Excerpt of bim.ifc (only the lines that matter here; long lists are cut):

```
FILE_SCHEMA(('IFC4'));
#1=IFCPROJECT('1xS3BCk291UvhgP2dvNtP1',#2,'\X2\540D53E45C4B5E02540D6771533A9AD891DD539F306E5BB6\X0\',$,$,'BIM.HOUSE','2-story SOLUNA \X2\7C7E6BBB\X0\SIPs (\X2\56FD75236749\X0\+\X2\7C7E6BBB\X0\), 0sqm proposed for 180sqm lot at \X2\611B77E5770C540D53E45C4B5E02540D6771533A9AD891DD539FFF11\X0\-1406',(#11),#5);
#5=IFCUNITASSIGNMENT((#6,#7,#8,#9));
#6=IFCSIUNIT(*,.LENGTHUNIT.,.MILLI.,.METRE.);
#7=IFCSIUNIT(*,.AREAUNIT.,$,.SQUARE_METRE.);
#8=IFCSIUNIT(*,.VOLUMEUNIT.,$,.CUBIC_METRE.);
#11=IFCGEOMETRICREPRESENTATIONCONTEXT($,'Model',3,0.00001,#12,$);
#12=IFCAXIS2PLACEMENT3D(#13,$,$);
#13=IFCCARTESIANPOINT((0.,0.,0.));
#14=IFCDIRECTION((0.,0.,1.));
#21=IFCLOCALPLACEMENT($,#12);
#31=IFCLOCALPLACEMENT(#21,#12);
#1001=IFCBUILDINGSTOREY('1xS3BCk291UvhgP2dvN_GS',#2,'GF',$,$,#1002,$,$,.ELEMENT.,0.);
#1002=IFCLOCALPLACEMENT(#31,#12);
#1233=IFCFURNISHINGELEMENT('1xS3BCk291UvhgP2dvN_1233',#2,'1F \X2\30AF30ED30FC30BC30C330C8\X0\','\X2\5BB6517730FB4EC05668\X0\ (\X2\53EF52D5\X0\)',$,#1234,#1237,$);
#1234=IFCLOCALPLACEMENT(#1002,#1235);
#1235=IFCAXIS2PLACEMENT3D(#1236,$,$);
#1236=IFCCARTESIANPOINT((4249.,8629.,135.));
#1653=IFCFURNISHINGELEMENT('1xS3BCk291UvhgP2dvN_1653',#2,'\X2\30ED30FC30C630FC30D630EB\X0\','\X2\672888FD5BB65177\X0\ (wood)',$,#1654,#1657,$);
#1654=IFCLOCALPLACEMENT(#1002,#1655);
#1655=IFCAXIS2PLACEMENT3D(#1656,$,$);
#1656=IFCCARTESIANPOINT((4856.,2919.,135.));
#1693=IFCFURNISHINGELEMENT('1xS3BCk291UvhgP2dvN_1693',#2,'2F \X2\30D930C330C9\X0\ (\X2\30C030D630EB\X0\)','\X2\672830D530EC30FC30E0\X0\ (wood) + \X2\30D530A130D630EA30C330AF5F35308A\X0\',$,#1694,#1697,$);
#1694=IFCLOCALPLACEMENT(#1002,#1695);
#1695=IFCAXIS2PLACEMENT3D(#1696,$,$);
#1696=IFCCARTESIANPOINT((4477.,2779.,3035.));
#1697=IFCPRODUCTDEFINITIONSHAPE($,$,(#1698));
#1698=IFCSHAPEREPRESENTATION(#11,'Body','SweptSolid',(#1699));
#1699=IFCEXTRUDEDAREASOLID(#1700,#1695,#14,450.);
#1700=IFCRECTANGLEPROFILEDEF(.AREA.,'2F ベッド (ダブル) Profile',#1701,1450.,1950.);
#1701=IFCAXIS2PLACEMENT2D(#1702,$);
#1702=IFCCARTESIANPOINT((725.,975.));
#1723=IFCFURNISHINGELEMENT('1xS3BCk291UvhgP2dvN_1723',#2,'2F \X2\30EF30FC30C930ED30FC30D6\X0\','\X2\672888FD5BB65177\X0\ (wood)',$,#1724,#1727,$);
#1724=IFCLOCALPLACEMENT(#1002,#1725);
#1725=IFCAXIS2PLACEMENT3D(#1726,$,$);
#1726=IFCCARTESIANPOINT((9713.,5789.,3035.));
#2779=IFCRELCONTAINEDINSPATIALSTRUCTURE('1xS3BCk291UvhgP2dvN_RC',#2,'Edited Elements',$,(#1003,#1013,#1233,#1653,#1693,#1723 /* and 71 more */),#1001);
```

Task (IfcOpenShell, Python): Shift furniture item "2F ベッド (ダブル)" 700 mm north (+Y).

```python
import ifcopenshell
import ifcopenshell.api.geometry
import ifcopenshell.util.placement
import ifcopenshell.util.unit

model = ifcopenshell.open("bim.ifc")
unit_scale = ifcopenshell.util.unit.calculate_unit_scale(model)

item = model.by_id(1693)
matrix = ifcopenshell.util.placement.get_local_placement(item.ObjectPlacement)
matrix[1, 3] += 0.7 / unit_scale
ifcopenshell.api.geometry.edit_object_placement(model, product=item, matrix=matrix, is_si=False)

print(ifcopenshell.util.placement.get_local_placement(item.ObjectPlacement).round(3) + 0.0)

model.write("bim_updated.ifc")
```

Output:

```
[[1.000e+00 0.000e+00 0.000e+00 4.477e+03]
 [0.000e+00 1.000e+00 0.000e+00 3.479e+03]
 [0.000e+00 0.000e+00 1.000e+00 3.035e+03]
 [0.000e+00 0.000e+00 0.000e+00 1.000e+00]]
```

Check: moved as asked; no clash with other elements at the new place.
